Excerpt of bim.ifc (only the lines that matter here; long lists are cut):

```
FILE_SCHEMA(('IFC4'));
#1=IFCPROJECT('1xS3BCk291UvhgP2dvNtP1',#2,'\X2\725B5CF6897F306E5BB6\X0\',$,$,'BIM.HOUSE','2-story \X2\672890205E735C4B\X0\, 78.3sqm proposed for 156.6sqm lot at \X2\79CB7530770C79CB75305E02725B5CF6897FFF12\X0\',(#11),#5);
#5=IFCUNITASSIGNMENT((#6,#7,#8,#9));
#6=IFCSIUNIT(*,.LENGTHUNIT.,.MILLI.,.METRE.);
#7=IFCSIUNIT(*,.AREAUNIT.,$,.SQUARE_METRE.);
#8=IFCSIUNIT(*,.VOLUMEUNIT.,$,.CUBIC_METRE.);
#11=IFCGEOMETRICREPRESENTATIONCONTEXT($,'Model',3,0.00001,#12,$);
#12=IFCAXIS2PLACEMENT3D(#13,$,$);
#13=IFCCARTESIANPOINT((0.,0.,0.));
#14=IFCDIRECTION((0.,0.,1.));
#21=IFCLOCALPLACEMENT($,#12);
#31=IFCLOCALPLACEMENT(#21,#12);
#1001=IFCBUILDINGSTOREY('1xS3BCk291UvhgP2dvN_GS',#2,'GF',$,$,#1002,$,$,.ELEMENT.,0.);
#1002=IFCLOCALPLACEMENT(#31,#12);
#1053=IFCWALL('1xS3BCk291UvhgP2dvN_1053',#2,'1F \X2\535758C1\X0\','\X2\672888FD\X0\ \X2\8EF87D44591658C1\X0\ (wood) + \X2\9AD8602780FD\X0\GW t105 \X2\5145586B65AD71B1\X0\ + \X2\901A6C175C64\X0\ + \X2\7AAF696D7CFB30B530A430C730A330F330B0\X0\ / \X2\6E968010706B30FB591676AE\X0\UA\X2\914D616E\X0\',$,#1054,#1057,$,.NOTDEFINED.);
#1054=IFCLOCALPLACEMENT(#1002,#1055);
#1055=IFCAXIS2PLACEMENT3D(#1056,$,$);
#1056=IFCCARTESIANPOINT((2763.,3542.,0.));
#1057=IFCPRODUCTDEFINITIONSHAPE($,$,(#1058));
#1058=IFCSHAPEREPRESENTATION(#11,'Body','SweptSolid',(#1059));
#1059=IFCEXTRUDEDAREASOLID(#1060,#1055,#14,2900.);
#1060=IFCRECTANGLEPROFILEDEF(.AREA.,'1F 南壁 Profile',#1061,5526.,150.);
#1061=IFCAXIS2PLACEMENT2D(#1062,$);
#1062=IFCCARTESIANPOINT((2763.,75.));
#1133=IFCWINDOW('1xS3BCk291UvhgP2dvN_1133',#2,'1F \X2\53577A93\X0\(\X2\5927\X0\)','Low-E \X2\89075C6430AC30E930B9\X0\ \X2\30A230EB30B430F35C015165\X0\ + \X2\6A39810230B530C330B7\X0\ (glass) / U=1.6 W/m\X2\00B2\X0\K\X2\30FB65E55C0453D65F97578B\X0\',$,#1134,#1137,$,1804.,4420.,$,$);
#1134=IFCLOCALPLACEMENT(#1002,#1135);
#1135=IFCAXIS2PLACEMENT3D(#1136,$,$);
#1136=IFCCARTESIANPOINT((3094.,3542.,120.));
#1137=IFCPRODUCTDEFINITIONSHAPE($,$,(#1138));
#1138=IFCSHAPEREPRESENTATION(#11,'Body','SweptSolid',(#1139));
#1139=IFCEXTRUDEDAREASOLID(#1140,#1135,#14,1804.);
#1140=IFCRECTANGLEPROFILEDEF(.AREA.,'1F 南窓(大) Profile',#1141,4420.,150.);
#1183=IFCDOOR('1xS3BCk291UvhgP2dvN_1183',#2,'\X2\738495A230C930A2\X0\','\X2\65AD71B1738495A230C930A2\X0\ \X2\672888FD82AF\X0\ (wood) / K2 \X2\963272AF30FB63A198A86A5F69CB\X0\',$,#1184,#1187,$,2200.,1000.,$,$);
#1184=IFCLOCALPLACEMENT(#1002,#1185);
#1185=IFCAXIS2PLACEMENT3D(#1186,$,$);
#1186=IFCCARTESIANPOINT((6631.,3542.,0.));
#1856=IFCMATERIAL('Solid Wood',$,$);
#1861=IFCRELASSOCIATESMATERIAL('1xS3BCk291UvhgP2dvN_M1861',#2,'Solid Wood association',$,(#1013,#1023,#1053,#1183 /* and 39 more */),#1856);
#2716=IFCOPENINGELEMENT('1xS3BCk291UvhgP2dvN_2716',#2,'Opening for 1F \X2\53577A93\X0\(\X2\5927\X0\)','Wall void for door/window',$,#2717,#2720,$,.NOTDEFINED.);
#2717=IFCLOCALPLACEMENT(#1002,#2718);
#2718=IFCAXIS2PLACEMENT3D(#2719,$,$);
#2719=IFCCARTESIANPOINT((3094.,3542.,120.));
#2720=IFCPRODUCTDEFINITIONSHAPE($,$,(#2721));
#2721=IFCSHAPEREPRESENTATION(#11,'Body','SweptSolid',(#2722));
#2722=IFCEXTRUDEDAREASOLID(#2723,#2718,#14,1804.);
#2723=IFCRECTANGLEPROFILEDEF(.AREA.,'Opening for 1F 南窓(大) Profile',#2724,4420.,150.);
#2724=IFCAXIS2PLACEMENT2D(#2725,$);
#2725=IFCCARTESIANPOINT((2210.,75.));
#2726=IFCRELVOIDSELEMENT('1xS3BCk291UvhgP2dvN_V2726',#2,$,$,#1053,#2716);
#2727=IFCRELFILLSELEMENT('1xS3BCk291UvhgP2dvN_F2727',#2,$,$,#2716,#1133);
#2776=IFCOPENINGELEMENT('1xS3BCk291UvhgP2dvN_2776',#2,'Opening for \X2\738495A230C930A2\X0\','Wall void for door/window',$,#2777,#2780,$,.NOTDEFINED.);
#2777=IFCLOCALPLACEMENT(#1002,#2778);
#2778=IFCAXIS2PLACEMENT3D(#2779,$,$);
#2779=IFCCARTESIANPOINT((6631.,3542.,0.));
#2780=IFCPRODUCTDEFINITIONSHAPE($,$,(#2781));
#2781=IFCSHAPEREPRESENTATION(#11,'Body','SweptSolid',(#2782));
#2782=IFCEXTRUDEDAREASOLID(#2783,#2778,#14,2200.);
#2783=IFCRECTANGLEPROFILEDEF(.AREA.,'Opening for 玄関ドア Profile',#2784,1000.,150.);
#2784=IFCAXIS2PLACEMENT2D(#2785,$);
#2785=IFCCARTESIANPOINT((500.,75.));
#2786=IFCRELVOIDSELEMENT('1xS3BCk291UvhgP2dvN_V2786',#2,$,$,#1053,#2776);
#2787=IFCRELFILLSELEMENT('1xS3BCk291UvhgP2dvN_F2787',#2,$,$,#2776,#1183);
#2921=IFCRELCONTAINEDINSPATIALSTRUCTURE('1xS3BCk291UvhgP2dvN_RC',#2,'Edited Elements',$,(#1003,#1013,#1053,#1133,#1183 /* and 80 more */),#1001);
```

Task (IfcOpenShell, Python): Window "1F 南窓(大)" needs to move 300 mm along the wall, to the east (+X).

```python
import ifcopenshell
import ifcopenshell.api.geometry
import ifcopenshell.util.placement

model = ifcopenshell.open("bim.ifc")

window = model.by_id(1133)
opening = window.FillsVoids[0].RelatingOpeningElement
wall = opening.VoidsElements[0].RelatingBuildingElement

wall_matrix = ifcopenshell.util.placement.get_local_placement(wall.ObjectPlacement)
shift = wall_matrix[:3, 0] * 300.0
before = ifcopenshell.util.placement.get_local_placement(window.ObjectPlacement)[:3, 3].copy()

# The window is not placed relative to its opening, so move both.
for product in (opening, window):
    matrix = ifcopenshell.util.placement.get_local_placement(product.ObjectPlacement)
    matrix[:3, 3] += shift
    ifcopenshell.api.geometry.edit_object_placement(model, product=product, matrix=matrix, is_si=False)

after = ifcopenshell.util.placement.get_local_placement(window.ObjectPlacement)[:3, 3]
print("window moved by", (after - before).round(3) + 0.0)

model.write("bim_rev.ifc")
```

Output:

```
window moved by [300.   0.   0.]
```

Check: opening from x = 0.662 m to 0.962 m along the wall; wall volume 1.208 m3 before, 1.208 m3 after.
